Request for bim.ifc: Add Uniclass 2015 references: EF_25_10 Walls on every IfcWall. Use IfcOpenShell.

First a look at what the model holds.

```python
import ifcopenshell

model = ifcopenshell.open("bim.ifc")
print(model.schema)
print("classifications:", [c.Name for c in model.by_type("IfcClassification")])
for ifc_class in ("IfcDoor", "IfcRoof", "IfcStair", "IfcWall", "IfcWindow"):
    print(ifc_class, len(model.by_type(ifc_class)))
```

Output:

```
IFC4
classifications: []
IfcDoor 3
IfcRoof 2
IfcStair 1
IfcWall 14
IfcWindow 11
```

```python
import ifcopenshell
import ifcopenshell.api.classification

model = ifcopenshell.open("bim.ifc")

system = ifcopenshell.api.classification.add_classification(model, classification="Uniclass 2015")

codes = {
    "IfcWall": ("EF_25_10", "Walls"),
}
for ifc_class, (code, name) in codes.items():
    products = model.by_type(ifc_class)
    ifcopenshell.api.classification.add_reference(
        model, products=products, classification=system, identification=code, name=name
    )
    print(code, len(products))

model.write("bim_v2.ifc")
```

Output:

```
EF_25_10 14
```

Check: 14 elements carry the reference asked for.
